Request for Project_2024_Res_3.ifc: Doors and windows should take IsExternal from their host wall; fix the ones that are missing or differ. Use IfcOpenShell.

First a look at what the model holds.

```python
import ifcopenshell
import ifcopenshell.util.element

model = ifcopenshell.open("Project_2024_Res_3.ifc")
print(model.schema)
seen = {}
for e in model.by_type("IfcDoor") + model.by_type("IfcWindow"):
    if not e.FillsVoids:
        continue
    host = e.FillsVoids[0].RelatingOpeningElement.VoidsElements[0].RelatingBuildingElement
    own = ifcopenshell.util.element.get_pset(e, f"Pset_{e.is_a()[3:].removesuffix('StandardCase')}Common", "IsExternal")
    wall = ifcopenshell.util.element.get_pset(host, "Pset_WallCommon", "IsExternal")
    seen[e.is_a(), own, wall] = seen.get((e.is_a(), own, wall), 0) + 1
for (cls, own, wall), count in sorted(seen.items(), key=str):
    print(count, cls, "IsExternal:", own, "| host wall:", wall)
```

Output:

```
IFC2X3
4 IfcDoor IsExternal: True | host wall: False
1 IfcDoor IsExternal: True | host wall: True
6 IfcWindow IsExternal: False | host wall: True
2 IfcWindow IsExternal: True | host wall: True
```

```python
import ifcopenshell
import ifcopenshell.api.pset
import ifcopenshell.util.element

model = ifcopenshell.open("Project_2024_Res_3.ifc")

count = 0
for ifc_class, pset_name in (("IfcDoor", "Pset_DoorCommon"), ("IfcWindow", "Pset_WindowCommon")):
    for e in model.by_type(ifc_class):
        if not e.FillsVoids:
            continue
        host = e.FillsVoids[0].RelatingOpeningElement.VoidsElements[0].RelatingBuildingElement
        external = ifcopenshell.util.element.get_pset(host, "Pset_WallCommon", "IsExternal")
        if external is None or ifcopenshell.util.element.get_pset(e, pset_name, "IsExternal") == external:
            continue
        pset = ifcopenshell.api.pset.add_pset(model, product=e, name=pset_name)
        ifcopenshell.api.pset.edit_pset(model, pset=pset, properties={"IsExternal": external})
        count += 1

print(count, "updated")

model.write("Project_2024_Res_3-out.ifc")
```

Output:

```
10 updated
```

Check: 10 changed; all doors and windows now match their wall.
